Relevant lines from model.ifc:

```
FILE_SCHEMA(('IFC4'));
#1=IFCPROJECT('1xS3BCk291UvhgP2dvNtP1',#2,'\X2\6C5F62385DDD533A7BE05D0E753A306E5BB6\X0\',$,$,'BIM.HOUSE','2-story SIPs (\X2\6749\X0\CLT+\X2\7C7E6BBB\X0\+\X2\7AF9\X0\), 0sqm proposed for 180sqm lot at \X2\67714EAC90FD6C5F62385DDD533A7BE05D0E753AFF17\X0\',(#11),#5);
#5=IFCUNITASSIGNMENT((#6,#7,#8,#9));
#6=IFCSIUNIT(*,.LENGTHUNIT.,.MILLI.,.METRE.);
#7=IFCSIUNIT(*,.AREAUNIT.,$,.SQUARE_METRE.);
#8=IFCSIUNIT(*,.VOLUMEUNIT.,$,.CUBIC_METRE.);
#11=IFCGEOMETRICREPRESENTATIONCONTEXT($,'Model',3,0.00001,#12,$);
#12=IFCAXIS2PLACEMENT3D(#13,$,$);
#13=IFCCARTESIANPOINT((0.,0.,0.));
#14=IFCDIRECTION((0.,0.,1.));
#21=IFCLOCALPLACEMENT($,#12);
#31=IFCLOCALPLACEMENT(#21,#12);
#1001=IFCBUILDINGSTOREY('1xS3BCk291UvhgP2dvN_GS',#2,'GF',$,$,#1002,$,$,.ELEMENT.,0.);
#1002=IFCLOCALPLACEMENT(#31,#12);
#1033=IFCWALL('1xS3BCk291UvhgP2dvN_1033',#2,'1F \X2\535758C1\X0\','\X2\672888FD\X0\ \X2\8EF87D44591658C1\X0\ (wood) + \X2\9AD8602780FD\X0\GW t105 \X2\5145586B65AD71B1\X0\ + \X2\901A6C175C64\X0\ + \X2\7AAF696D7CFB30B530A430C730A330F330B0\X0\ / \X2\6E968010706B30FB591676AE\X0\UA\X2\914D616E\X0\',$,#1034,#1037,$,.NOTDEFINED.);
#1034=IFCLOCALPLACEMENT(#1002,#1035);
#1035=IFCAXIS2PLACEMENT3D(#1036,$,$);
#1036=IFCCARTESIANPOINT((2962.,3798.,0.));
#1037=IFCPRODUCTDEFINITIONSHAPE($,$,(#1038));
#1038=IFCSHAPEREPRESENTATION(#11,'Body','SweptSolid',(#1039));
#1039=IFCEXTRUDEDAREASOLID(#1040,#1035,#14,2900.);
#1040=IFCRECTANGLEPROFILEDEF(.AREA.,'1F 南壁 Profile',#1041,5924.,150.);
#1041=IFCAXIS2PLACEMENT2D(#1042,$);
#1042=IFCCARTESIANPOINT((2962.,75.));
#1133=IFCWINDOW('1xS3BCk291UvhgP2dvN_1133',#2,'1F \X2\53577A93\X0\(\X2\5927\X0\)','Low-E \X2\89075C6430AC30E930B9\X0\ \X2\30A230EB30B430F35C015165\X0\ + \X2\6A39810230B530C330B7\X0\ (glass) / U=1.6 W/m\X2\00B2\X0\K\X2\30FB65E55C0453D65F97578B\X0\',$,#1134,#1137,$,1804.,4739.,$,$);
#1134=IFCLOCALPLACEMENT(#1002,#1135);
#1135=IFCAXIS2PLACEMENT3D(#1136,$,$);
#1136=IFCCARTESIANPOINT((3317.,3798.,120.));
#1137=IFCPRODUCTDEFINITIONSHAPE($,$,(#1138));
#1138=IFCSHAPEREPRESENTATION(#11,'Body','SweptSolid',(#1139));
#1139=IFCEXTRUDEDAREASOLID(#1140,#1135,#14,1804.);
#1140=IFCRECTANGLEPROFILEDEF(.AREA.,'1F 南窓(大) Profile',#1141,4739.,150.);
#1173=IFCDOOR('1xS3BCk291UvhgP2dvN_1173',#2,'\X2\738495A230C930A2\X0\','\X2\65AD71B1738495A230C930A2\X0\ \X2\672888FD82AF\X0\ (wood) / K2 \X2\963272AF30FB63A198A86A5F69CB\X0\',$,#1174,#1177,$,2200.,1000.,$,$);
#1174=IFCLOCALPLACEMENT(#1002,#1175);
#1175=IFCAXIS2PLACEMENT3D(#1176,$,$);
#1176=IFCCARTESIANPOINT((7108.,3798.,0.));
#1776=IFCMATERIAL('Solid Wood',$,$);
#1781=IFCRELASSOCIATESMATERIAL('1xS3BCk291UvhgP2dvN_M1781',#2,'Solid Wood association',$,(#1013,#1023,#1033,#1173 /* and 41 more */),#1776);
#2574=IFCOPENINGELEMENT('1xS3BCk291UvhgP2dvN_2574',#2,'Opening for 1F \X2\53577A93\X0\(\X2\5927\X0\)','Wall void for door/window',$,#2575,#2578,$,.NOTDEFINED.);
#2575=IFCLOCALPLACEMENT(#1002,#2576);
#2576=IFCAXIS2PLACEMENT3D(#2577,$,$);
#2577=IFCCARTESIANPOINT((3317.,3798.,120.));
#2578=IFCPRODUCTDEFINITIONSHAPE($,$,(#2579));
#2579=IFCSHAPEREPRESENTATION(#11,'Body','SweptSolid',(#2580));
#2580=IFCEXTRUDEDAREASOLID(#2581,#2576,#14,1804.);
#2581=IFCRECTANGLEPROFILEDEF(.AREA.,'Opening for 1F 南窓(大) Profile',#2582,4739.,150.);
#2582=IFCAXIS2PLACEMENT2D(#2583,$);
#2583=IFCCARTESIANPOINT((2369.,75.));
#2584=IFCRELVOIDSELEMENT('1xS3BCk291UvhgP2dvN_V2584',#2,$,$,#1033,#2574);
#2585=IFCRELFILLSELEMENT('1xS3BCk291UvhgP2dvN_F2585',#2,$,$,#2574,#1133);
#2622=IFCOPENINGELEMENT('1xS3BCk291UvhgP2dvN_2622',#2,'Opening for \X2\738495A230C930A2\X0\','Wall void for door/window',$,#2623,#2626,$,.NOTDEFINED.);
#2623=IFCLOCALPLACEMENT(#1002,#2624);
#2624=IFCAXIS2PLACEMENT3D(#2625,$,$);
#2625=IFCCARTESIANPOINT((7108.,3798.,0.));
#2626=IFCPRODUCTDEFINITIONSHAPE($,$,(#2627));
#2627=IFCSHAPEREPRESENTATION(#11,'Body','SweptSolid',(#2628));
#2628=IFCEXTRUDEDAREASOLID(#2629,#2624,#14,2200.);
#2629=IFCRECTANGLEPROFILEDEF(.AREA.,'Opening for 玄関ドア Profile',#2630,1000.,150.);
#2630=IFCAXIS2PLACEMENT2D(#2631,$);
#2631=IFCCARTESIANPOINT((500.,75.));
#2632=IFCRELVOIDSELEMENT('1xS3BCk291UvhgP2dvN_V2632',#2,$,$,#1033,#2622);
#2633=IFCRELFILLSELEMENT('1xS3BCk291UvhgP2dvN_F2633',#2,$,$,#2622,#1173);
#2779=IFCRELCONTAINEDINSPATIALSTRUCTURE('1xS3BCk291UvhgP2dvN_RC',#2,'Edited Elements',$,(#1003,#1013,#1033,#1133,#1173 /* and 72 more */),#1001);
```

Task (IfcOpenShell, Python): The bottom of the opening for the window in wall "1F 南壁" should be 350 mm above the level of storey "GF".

```python
import numpy as np
import ifcopenshell
import ifcopenshell.api.geometry
import ifcopenshell.geom
import ifcopenshell.util.element
import ifcopenshell.util.placement
import ifcopenshell.util.shape
import ifcopenshell.util.unit

model = ifcopenshell.open("model.ifc")
unit_scale = ifcopenshell.util.unit.calculate_unit_scale(model)

window = model.by_guid("1xS3BCk291UvhgP2dvN_1133")
opening = window.FillsVoids[0].RelatingOpeningElement
storey = ifcopenshell.util.element.get_container(window, ifc_class="IfcBuildingStorey")
level = ifcopenshell.util.placement.get_local_placement(storey.ObjectPlacement)[2, 3]

# The opening's origin need not be at the sill, so measure its lowest point.
shape = ifcopenshell.geom.create_shape(ifcopenshell.geom.settings(), opening)
bottom = ifcopenshell.util.shape.get_shape_bottom_elevation(shape, shape.geometry) / unit_scale
dz = level + 0.35 / unit_scale - bottom

shift = np.array([0.0, 0.0, dz])
# The window is not placed relative to its opening, so move both.
for product in (opening, window):
    matrix = ifcopenshell.util.placement.get_local_placement(product.ObjectPlacement)
    matrix[:3, 3] += shift
    ifcopenshell.api.geometry.edit_object_placement(model, product=product, matrix=matrix, is_si=False)

print(f"moved by {dz * unit_scale:+.3f} m")

model.write("model-out.ifc")
```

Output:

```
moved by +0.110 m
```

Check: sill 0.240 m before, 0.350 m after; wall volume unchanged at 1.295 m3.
